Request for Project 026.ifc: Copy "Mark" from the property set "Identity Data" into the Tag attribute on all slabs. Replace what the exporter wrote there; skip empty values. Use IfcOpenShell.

First a look at what the model holds.

```python
import ifcopenshell
import ifcopenshell.util.element

model = ifcopenshell.open("Project 026.ifc")
print(model.schema)
slabs = model.by_type("IfcSlab")
print(len(slabs), "slabs")
for e in slabs[:8]:
    source = ifcopenshell.util.element.get_pset(e, "Identity Data", "Mark")
    target = e.Tag
    print(e.id(), repr(source), repr(target), sep=" | ")
```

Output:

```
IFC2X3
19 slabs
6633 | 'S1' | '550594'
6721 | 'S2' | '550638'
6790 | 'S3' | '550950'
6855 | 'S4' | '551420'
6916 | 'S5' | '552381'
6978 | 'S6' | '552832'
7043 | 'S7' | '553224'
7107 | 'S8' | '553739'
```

```python
import ifcopenshell
import ifcopenshell.util.element

model = ifcopenshell.open("Project 026.ifc")

count = 0
for e in model.by_type("IfcSlab"):
    value = ifcopenshell.util.element.get_pset(e, "Identity Data", "Mark")
    current = e.Tag
    if not value or not value.strip() or current == value:
        continue
    e.Tag = value
    count += 1

print(count, "slabs updated")

model.write("Project 026_edited.ifc")
```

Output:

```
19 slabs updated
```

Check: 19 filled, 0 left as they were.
